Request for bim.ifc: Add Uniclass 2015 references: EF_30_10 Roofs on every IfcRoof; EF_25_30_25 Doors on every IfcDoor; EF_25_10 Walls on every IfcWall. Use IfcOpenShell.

First a look at what the model holds.

```python
import ifcopenshell

model = ifcopenshell.open("bim.ifc")
print(model.schema)
print("classifications:", [c.Name for c in model.by_type("IfcClassification")])
for ifc_class in ("IfcDoor", "IfcRoof", "IfcStair", "IfcWall", "IfcWindow"):
    print(ifc_class, len(model.by_type(ifc_class)))
```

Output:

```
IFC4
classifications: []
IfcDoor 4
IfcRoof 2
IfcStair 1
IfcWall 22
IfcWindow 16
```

```python
import ifcopenshell
import ifcopenshell.api.classification

model = ifcopenshell.open("bim.ifc")

system = ifcopenshell.api.classification.add_classification(model, classification="Uniclass 2015")

codes = {
    "IfcRoof": ("EF_30_10", "Roofs"),
    "IfcDoor": ("EF_25_30_25", "Doors"),
    "IfcWall": ("EF_25_10", "Walls"),
}
for ifc_class, (code, name) in codes.items():
    products = model.by_type(ifc_class)
    ifcopenshell.api.classification.add_reference(
        model, products=products, classification=system, identification=code, name=name
    )
    print(code, len(products))

model.write("bim-out.ifc")
```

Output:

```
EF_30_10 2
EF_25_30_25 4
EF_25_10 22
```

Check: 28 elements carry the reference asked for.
